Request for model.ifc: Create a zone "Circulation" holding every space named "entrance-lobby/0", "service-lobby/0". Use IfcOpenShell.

First a look at what the model holds.

```python
import ifcopenshell

model = ifcopenshell.open("model.ifc")
print(model.schema)
seen = {}
for space in model.by_type("IfcSpace"):
    seen[space.Name] = seen.get(space.Name, 0) + 1
for name, count in sorted(seen.items(), key=str):
    print(count, "x", name)
print("zones:", [z.Name for z in model.by_type("IfcZone")][:20])
```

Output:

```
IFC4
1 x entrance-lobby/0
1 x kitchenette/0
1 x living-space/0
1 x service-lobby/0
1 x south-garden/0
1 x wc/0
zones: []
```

```python
import ifcopenshell
import ifcopenshell.api.group
import ifcopenshell.api.root

model = ifcopenshell.open("model.ifc")

names = {"entrance-lobby/0", "service-lobby/0"}
spaces = [s for s in model.by_type("IfcSpace") if s.Name in names]

zone = ifcopenshell.api.root.create_entity(model, ifc_class="IfcZone", name="Circulation")
ifcopenshell.api.group.assign_group(model, products=spaces, group=zone)
print(len(spaces), "spaces in", zone.Name)

model.write("model_v2.ifc")
```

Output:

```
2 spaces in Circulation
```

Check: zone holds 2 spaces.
